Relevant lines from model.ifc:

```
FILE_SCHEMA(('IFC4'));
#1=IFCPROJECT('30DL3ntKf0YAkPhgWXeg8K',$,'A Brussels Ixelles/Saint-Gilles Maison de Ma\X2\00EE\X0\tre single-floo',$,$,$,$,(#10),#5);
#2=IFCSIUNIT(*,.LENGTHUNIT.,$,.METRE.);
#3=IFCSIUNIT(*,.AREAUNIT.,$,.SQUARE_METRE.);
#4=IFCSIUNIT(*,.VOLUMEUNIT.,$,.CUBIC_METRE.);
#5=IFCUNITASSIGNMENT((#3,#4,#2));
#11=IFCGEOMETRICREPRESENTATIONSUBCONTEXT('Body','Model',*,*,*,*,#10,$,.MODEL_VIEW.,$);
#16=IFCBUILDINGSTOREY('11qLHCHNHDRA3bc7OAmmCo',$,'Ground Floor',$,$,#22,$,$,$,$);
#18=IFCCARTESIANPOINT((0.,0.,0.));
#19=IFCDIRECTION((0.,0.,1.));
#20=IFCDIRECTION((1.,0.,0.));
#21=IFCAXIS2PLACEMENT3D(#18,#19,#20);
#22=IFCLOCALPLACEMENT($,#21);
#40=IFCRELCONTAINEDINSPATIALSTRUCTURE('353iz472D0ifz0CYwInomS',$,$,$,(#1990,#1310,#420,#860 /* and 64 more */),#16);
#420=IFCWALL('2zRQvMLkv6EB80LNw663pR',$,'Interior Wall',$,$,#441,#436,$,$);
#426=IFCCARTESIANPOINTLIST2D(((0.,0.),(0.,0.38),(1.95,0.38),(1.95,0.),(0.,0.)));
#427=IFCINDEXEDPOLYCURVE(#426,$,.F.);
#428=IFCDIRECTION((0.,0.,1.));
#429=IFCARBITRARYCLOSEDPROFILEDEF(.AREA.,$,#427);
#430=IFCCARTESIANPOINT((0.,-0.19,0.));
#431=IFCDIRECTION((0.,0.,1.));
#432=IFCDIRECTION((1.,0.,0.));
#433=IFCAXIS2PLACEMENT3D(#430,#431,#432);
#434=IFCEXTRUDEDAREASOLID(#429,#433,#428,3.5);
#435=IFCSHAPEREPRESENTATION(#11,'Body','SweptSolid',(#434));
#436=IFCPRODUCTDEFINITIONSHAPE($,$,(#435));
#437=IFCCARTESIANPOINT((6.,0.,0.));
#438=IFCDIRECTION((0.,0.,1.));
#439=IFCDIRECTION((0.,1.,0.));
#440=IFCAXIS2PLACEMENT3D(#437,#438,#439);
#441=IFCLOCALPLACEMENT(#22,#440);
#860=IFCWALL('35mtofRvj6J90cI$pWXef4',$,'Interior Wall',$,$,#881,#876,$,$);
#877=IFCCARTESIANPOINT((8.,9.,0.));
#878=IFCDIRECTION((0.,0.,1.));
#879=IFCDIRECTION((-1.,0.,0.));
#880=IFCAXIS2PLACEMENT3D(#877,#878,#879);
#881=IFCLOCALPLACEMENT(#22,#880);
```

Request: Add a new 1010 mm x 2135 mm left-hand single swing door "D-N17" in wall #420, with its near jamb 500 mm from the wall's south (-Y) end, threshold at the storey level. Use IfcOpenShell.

```python
import numpy as np
import ifcopenshell
import ifcopenshell.api.feature
import ifcopenshell.api.geometry
import ifcopenshell.api.root
import ifcopenshell.api.spatial
import ifcopenshell.geom
import ifcopenshell.util.element
import ifcopenshell.util.placement
import ifcopenshell.util.representation
import ifcopenshell.util.shape
import ifcopenshell.util.unit

model = ifcopenshell.open("model.ifc")
unit_scale = ifcopenshell.util.unit.calculate_unit_scale(model)
settings = ifcopenshell.geom.settings()


def volume(element):
    """Net volume in cubic metres, openings subtracted."""
    shape = ifcopenshell.geom.create_shape(settings, element)
    return ifcopenshell.util.shape.get_volume(shape.geometry)


wall = model.by_id(420)
storey = ifcopenshell.util.element.get_container(wall, ifc_class="IfcBuildingStorey")
context = ifcopenshell.util.representation.get_context(model, "Model", "Body", "MODEL_VIEW")
before = volume(wall)

width, height, from_end, sill = 1.01, 2.135, 0.5, 0.0  # metres

# The wall runs along its own X axis, and the end named is its -X end.
wall_shape = ifcopenshell.geom.create_shape(settings, wall)
x, y, z = ifcopenshell.util.shape.get_vertices(wall_shape.geometry).T
start = x.min() + from_end
face, thickness = float(y.min()), float(y.max() - y.min())
wall_matrix = ifcopenshell.util.placement.get_local_placement(wall.ObjectPlacement)
level = ifcopenshell.util.placement.get_local_placement(storey.ObjectPlacement)[2, 3]


def in_wall(x, y):
    """Placement at x, y metres in the wall's axes, at sill height."""
    matrix = wall_matrix.copy()
    matrix[:, 3] = wall_matrix @ np.array([x / unit_scale, y / unit_scale, 0.0, 1.0])
    matrix[2, 3] = level + sill / unit_scale
    return matrix


# Opening: a box that overshoots both wall faces by 50 mm.
opening = ifcopenshell.api.root.create_entity(model, ifc_class="IfcOpeningElement", predefined_type="OPENING")
box = ifcopenshell.api.geometry.add_wall_representation(
    model, context=context, length=width, height=height, thickness=thickness + 0.1
)
ifcopenshell.api.geometry.assign_representation(model, product=opening, representation=box)
ifcopenshell.api.geometry.edit_object_placement(model, product=opening, matrix=in_wall(start, face - 0.05), is_si=False)
ifcopenshell.api.feature.add_feature(model, feature=opening, element=wall)

door = ifcopenshell.api.root.create_entity(model, ifc_class="IfcDoor", name="D-N17", predefined_type="DOOR")
door.OverallWidth, door.OverallHeight = width / unit_scale, height / unit_scale
door.OperationType = "SINGLE_SWING_LEFT"
body = ifcopenshell.api.geometry.add_door_representation(
    model,
    context=context,
    overall_width=door.OverallWidth,
    overall_height=door.OverallHeight,
    operation_type="SINGLE_SWING_LEFT",
    lining_properties={"LiningDepth": thickness / unit_scale, "ThresholdDepth": thickness / unit_scale},
)
ifcopenshell.api.geometry.assign_representation(model, product=door, representation=body)
ifcopenshell.api.spatial.assign_container(model, products=[door], relating_structure=storey)
ifcopenshell.api.feature.add_filling(model, opening=opening, element=door)

# The lining spans the wall, so the door starts at the wall face.
ifcopenshell.api.geometry.edit_object_placement(model, product=door, matrix=in_wall(start, face), is_si=False)

after = volume(wall)

print(f"wall volume {before:.3f} -> {after:.3f} m3")

model.write("model_edited.ifc")
```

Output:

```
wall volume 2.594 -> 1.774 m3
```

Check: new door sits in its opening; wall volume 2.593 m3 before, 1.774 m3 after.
